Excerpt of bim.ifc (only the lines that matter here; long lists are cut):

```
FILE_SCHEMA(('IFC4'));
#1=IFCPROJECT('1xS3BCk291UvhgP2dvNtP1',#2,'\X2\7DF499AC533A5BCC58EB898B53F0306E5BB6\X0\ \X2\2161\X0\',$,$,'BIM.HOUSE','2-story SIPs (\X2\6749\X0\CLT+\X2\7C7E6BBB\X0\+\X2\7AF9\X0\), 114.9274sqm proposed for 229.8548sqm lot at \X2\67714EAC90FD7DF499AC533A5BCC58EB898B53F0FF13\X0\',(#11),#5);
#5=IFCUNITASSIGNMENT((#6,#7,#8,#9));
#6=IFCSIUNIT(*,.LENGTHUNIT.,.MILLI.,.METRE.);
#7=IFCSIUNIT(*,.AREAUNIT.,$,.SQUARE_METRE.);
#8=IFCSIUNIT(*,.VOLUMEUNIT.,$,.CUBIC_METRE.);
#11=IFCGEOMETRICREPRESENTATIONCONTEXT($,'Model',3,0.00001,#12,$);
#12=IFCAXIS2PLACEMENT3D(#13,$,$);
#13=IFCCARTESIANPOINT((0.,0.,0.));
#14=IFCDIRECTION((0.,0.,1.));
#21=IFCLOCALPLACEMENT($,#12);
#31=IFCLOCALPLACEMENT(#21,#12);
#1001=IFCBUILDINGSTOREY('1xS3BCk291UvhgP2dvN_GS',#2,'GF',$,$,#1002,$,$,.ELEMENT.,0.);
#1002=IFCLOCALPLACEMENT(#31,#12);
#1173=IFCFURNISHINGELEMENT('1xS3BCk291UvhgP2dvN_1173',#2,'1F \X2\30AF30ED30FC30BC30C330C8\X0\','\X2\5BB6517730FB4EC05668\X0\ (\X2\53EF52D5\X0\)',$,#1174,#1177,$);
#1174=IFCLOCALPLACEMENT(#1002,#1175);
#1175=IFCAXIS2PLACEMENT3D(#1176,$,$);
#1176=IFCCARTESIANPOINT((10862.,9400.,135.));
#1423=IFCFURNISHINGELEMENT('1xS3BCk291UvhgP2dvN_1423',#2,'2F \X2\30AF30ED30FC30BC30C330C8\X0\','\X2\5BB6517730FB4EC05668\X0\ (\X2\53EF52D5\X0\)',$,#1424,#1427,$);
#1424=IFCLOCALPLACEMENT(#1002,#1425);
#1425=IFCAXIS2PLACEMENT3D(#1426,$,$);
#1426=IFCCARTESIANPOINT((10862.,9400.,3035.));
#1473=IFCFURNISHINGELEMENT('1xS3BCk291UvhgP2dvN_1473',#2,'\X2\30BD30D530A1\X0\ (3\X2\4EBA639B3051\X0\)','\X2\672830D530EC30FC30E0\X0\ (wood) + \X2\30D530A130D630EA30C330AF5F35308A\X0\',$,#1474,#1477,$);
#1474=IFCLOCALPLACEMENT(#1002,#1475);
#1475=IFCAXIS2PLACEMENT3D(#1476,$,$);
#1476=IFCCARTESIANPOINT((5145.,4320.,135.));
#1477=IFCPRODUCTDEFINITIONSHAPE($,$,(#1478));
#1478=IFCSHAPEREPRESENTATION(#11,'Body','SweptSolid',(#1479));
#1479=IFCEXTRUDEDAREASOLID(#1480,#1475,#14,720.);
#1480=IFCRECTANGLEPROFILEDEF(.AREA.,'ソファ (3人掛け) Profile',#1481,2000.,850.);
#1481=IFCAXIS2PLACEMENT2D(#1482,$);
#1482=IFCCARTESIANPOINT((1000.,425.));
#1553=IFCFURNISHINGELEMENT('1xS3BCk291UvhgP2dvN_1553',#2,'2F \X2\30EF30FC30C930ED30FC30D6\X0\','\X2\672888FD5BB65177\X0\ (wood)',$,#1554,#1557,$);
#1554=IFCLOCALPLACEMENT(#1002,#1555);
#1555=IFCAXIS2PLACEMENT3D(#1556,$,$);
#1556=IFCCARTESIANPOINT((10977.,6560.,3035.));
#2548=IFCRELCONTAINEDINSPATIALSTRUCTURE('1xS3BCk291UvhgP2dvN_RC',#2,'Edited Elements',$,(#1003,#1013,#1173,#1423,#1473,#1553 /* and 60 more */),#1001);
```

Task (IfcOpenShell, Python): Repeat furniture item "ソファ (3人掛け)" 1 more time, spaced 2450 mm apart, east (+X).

```python
import numpy as np
import ifcopenshell
import ifcopenshell.api.geometry
import ifcopenshell.api.root
import ifcopenshell.util.element
import ifcopenshell.util.placement
import ifcopenshell.util.unit

model = ifcopenshell.open("bim.ifc")
unit_scale = ifcopenshell.util.unit.calculate_unit_scale(model)


def reuse_history(source, copy):
    """copy_class also copies each property set's owner history, people and application; keep the originals."""
    for rel in copy.IsDefinedBy:
        if rel.is_a("IfcRelDefinesByProperties") and (history := rel.RelatingPropertyDefinition.OwnerHistory):
            rel.RelatingPropertyDefinition.OwnerHistory = source.OwnerHistory
            ifcopenshell.util.element.remove_deep2(model, history)


source = model.by_guid("1xS3BCk291UvhgP2dvN_1473")
base = ifcopenshell.util.placement.get_local_placement(source.ObjectPlacement)
step = np.array([1.0, 0.0, 0.0]) * 2.45 / unit_scale

for i in range(1, 2):
    copy = ifcopenshell.api.root.copy_class(model, product=source)
    copy.Representation = ifcopenshell.util.element.copy_deep(
        model, source.Representation, exclude=["IfcGeometricRepresentationContext", "IfcRepresentationMap"]
    )
    reuse_history(source, copy)
    matrix = base.copy()
    matrix[:3, 3] += i * step
    print("added at", matrix[:3, 3].round(3) + 0.0)
    ifcopenshell.api.geometry.edit_object_placement(model, product=copy, matrix=matrix, is_si=False)

model.write("bim_edited.ifc")
```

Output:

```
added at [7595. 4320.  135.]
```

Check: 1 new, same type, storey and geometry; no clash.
